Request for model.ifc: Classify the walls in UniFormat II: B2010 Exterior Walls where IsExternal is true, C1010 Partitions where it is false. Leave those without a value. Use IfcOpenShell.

First a look at what the model holds.

```python
import ifcopenshell
import ifcopenshell.util.element

model = ifcopenshell.open("model.ifc")
print(model.schema)
print("classifications:", [c.Name for c in model.by_type("IfcClassification")])
values = [ifcopenshell.util.element.get_pset(e, "Pset_WallCommon", "IsExternal") for e in model.by_type("IfcWall")]
for value in (True, False, None):
    print("IsExternal", value, values.count(value))
```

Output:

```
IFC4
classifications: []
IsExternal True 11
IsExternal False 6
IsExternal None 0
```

```python
import ifcopenshell
import ifcopenshell.api.classification
import ifcopenshell.util.element

model = ifcopenshell.open("model.ifc")

system = ifcopenshell.api.classification.add_classification(model, classification="UniFormat II")

walls = model.by_type("IfcWall")
external = {e: ifcopenshell.util.element.get_pset(e, "Pset_WallCommon", "IsExternal") for e in walls}
for flag, code, name in ((True, "B2010", "Exterior Walls"), (False, "C1010", "Partitions")):
    products = [e for e in walls if external[e] is flag]
    ifcopenshell.api.classification.add_reference(
        model, products=products, classification=system, identification=code, name=name
    )
    print(code, len(products))

model.write("model_v2.ifc")
```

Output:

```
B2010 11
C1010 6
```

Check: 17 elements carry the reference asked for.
